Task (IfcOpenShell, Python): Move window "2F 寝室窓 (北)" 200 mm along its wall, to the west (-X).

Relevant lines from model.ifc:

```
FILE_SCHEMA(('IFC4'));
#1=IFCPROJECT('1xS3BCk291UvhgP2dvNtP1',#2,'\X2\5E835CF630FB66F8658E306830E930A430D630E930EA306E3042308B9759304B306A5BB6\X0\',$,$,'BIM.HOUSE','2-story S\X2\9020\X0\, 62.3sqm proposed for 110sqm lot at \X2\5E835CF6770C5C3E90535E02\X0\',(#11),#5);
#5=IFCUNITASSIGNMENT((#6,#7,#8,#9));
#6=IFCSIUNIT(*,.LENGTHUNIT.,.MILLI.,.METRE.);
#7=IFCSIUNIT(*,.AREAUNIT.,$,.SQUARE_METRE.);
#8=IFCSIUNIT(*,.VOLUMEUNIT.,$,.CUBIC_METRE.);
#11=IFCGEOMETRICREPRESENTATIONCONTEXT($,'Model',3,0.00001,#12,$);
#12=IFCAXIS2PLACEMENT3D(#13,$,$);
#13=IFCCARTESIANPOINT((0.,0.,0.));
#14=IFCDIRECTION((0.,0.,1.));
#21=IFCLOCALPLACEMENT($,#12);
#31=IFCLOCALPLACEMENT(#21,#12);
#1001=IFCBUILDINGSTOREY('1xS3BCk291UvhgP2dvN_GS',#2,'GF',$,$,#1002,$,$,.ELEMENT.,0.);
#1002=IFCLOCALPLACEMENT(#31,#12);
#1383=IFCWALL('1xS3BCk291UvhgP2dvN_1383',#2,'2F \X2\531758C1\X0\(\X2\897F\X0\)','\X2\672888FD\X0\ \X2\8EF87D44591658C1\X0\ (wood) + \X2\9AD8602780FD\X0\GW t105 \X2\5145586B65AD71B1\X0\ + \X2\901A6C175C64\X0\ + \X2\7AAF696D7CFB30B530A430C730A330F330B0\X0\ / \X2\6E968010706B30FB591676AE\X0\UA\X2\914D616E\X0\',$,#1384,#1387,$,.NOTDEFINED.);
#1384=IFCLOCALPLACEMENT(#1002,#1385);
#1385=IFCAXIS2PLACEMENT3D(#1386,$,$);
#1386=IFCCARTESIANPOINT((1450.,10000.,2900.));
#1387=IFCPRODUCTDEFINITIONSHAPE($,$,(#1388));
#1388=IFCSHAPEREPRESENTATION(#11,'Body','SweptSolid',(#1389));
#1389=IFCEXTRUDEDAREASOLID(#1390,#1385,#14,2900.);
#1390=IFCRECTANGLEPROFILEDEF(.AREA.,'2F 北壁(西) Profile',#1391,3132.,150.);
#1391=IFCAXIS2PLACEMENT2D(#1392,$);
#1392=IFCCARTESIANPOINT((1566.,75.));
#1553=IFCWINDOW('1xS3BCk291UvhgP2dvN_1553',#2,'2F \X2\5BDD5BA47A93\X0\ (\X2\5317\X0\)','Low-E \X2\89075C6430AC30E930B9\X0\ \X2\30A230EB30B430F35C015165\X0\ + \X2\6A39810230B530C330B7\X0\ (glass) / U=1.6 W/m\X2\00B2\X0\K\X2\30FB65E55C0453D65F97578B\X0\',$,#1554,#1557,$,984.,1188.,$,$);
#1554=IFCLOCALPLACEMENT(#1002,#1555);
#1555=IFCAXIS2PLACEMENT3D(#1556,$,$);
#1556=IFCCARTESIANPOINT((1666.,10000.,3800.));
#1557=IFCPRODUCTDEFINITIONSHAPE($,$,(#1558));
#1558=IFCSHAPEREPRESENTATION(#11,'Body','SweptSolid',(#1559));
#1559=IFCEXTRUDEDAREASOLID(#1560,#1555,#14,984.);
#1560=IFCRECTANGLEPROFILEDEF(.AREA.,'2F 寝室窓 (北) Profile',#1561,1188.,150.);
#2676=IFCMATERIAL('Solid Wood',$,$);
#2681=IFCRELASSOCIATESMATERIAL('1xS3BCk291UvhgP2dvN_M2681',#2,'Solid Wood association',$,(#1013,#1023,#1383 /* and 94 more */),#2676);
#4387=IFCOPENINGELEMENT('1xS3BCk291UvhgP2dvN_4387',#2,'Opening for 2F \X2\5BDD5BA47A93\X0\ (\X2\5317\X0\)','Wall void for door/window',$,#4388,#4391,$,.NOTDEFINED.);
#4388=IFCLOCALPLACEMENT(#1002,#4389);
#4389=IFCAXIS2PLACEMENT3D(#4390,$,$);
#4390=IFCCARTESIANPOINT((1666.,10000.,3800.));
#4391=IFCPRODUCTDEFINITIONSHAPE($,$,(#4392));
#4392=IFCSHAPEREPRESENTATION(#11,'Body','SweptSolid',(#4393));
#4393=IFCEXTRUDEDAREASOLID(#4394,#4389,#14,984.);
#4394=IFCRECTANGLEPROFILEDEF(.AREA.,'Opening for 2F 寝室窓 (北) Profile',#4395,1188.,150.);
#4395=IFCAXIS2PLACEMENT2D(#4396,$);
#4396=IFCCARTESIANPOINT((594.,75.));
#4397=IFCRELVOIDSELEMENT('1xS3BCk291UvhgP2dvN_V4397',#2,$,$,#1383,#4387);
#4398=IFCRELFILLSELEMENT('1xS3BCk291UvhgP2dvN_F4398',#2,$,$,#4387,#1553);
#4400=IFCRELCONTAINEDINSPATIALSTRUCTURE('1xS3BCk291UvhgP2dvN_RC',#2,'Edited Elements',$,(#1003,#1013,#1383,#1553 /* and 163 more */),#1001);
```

```python
import ifcopenshell
import ifcopenshell.api.geometry
import ifcopenshell.util.placement
import ifcopenshell.util.unit

model = ifcopenshell.open("model.ifc")
unit_scale = ifcopenshell.util.unit.calculate_unit_scale(model)

window = model.by_guid("1xS3BCk291UvhgP2dvN_1553")
opening = window.FillsVoids[0].RelatingOpeningElement
wall = opening.VoidsElements[0].RelatingBuildingElement

wall_matrix = ifcopenshell.util.placement.get_local_placement(wall.ObjectPlacement)
shift = wall_matrix[:3, 0] * -0.2 / unit_scale
before = ifcopenshell.util.placement.get_local_placement(window.ObjectPlacement)[:3, 3].copy()

# The window is not placed relative to its opening, so move both.
for product in (opening, window):
    matrix = ifcopenshell.util.placement.get_local_placement(product.ObjectPlacement)
    matrix[:3, 3] += shift
    ifcopenshell.api.geometry.edit_object_placement(model, product=product, matrix=matrix, is_si=False)

after = ifcopenshell.util.placement.get_local_placement(window.ObjectPlacement)[:3, 3]
print("window moved by", (after - before).round(3) + 0.0)

model.write("model_edited.ifc")
```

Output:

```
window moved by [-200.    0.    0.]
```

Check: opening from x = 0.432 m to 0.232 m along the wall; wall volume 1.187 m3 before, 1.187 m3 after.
